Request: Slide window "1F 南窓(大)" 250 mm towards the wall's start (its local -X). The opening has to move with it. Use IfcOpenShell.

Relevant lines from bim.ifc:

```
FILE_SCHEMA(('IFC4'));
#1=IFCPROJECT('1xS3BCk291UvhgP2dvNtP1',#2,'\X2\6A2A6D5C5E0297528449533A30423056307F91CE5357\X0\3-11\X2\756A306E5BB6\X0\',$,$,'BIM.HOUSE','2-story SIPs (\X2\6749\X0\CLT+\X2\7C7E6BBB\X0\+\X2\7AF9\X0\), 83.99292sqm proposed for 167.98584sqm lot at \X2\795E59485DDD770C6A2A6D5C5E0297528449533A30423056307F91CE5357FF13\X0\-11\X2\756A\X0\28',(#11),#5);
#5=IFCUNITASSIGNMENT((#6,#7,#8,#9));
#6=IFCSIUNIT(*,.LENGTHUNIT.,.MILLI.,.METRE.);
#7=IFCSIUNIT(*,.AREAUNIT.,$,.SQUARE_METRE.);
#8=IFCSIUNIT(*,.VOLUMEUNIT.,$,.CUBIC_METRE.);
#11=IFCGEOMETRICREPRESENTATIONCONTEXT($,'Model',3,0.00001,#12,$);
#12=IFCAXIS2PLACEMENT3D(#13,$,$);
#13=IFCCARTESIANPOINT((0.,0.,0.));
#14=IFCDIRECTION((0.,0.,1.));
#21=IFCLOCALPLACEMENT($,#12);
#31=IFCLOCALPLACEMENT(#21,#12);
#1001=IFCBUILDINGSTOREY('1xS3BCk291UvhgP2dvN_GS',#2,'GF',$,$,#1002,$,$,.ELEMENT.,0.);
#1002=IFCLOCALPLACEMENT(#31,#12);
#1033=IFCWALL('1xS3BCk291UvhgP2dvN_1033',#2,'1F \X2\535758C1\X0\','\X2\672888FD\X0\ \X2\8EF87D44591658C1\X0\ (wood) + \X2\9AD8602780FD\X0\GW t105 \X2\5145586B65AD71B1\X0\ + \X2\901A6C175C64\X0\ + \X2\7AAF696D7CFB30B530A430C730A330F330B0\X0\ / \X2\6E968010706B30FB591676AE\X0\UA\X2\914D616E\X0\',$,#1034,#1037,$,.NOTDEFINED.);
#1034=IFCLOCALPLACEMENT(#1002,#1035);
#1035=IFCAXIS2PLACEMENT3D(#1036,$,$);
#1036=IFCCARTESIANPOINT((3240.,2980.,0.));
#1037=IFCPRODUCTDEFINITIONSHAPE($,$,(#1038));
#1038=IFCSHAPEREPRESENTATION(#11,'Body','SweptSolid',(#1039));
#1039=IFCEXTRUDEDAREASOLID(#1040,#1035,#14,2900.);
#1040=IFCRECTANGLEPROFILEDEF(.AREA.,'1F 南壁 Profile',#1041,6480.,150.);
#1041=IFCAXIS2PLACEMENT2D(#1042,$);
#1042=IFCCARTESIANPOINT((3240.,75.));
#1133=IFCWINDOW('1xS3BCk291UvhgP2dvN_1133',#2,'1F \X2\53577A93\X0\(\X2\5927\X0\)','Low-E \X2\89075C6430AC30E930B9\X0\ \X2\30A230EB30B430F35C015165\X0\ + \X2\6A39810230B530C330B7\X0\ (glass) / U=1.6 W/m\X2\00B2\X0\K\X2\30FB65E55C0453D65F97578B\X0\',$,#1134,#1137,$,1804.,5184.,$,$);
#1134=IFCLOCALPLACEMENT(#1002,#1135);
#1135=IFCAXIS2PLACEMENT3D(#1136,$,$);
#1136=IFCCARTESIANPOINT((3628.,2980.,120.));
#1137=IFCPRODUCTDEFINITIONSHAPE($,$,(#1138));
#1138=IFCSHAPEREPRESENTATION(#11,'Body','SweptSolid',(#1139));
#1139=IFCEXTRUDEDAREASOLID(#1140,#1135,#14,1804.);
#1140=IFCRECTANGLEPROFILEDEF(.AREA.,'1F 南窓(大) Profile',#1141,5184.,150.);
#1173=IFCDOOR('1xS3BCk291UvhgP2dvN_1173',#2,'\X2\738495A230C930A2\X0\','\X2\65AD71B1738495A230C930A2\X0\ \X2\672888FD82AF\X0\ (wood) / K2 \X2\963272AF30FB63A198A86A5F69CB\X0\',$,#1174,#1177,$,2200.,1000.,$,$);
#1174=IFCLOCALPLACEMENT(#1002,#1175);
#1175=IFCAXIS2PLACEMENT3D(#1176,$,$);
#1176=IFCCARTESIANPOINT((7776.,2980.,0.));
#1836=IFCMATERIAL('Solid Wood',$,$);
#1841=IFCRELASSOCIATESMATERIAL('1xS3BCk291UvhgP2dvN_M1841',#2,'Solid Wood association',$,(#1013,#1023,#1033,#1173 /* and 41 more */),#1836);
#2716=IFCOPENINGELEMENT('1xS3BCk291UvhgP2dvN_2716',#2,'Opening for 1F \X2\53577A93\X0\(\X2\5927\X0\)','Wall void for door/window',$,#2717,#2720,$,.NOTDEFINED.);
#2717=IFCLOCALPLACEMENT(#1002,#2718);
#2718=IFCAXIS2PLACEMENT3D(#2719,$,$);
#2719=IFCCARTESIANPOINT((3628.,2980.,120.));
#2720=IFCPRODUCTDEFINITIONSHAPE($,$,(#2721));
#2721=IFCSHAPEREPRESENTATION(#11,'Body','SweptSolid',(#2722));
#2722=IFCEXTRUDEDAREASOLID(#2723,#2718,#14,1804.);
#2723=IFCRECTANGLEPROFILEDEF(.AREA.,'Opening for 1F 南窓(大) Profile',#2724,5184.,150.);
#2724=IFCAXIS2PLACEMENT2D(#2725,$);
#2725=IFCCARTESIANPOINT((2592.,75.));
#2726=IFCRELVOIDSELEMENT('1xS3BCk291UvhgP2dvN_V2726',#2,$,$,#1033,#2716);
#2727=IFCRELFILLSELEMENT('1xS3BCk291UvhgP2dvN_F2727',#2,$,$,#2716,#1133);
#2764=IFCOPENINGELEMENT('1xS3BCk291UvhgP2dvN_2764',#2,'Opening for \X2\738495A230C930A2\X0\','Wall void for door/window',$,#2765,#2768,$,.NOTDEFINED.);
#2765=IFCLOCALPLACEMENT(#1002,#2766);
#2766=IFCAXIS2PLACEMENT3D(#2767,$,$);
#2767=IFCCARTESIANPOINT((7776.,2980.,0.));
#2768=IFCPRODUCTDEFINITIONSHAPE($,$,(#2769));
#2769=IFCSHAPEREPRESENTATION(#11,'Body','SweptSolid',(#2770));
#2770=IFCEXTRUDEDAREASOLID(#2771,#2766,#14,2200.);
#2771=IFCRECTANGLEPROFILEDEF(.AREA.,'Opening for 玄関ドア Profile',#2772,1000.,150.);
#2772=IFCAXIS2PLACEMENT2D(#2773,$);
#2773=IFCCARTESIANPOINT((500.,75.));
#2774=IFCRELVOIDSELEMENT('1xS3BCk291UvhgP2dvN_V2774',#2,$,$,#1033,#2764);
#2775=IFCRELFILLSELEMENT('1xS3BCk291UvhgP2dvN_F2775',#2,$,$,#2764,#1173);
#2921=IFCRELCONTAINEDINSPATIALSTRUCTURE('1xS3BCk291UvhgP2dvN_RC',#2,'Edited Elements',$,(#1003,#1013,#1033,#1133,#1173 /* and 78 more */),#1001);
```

```python
import ifcopenshell
import ifcopenshell.api.geometry
import ifcopenshell.util.placement

model = ifcopenshell.open("bim.ifc")

window = model.by_guid("1xS3BCk291UvhgP2dvN_1133")
opening = window.FillsVoids[0].RelatingOpeningElement
wall = opening.VoidsElements[0].RelatingBuildingElement

wall_matrix = ifcopenshell.util.placement.get_local_placement(wall.ObjectPlacement)
shift = wall_matrix[:3, 0] * -250.0
before = ifcopenshell.util.placement.get_local_placement(window.ObjectPlacement)[:3, 3].copy()

# The window is not placed relative to its opening, so move both.
for product in (opening, window):
    matrix = ifcopenshell.util.placement.get_local_placement(product.ObjectPlacement)
    matrix[:3, 3] += shift
    ifcopenshell.api.geometry.edit_object_placement(model, product=product, matrix=matrix, is_si=False)

after = ifcopenshell.util.placement.get_local_placement(window.ObjectPlacement)[:3, 3]
print("window moved by", (after - before).round(3) + 0.0)

model.write("bim_updated.ifc")
```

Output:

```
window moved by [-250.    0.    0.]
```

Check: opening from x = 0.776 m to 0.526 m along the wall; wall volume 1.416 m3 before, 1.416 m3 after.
